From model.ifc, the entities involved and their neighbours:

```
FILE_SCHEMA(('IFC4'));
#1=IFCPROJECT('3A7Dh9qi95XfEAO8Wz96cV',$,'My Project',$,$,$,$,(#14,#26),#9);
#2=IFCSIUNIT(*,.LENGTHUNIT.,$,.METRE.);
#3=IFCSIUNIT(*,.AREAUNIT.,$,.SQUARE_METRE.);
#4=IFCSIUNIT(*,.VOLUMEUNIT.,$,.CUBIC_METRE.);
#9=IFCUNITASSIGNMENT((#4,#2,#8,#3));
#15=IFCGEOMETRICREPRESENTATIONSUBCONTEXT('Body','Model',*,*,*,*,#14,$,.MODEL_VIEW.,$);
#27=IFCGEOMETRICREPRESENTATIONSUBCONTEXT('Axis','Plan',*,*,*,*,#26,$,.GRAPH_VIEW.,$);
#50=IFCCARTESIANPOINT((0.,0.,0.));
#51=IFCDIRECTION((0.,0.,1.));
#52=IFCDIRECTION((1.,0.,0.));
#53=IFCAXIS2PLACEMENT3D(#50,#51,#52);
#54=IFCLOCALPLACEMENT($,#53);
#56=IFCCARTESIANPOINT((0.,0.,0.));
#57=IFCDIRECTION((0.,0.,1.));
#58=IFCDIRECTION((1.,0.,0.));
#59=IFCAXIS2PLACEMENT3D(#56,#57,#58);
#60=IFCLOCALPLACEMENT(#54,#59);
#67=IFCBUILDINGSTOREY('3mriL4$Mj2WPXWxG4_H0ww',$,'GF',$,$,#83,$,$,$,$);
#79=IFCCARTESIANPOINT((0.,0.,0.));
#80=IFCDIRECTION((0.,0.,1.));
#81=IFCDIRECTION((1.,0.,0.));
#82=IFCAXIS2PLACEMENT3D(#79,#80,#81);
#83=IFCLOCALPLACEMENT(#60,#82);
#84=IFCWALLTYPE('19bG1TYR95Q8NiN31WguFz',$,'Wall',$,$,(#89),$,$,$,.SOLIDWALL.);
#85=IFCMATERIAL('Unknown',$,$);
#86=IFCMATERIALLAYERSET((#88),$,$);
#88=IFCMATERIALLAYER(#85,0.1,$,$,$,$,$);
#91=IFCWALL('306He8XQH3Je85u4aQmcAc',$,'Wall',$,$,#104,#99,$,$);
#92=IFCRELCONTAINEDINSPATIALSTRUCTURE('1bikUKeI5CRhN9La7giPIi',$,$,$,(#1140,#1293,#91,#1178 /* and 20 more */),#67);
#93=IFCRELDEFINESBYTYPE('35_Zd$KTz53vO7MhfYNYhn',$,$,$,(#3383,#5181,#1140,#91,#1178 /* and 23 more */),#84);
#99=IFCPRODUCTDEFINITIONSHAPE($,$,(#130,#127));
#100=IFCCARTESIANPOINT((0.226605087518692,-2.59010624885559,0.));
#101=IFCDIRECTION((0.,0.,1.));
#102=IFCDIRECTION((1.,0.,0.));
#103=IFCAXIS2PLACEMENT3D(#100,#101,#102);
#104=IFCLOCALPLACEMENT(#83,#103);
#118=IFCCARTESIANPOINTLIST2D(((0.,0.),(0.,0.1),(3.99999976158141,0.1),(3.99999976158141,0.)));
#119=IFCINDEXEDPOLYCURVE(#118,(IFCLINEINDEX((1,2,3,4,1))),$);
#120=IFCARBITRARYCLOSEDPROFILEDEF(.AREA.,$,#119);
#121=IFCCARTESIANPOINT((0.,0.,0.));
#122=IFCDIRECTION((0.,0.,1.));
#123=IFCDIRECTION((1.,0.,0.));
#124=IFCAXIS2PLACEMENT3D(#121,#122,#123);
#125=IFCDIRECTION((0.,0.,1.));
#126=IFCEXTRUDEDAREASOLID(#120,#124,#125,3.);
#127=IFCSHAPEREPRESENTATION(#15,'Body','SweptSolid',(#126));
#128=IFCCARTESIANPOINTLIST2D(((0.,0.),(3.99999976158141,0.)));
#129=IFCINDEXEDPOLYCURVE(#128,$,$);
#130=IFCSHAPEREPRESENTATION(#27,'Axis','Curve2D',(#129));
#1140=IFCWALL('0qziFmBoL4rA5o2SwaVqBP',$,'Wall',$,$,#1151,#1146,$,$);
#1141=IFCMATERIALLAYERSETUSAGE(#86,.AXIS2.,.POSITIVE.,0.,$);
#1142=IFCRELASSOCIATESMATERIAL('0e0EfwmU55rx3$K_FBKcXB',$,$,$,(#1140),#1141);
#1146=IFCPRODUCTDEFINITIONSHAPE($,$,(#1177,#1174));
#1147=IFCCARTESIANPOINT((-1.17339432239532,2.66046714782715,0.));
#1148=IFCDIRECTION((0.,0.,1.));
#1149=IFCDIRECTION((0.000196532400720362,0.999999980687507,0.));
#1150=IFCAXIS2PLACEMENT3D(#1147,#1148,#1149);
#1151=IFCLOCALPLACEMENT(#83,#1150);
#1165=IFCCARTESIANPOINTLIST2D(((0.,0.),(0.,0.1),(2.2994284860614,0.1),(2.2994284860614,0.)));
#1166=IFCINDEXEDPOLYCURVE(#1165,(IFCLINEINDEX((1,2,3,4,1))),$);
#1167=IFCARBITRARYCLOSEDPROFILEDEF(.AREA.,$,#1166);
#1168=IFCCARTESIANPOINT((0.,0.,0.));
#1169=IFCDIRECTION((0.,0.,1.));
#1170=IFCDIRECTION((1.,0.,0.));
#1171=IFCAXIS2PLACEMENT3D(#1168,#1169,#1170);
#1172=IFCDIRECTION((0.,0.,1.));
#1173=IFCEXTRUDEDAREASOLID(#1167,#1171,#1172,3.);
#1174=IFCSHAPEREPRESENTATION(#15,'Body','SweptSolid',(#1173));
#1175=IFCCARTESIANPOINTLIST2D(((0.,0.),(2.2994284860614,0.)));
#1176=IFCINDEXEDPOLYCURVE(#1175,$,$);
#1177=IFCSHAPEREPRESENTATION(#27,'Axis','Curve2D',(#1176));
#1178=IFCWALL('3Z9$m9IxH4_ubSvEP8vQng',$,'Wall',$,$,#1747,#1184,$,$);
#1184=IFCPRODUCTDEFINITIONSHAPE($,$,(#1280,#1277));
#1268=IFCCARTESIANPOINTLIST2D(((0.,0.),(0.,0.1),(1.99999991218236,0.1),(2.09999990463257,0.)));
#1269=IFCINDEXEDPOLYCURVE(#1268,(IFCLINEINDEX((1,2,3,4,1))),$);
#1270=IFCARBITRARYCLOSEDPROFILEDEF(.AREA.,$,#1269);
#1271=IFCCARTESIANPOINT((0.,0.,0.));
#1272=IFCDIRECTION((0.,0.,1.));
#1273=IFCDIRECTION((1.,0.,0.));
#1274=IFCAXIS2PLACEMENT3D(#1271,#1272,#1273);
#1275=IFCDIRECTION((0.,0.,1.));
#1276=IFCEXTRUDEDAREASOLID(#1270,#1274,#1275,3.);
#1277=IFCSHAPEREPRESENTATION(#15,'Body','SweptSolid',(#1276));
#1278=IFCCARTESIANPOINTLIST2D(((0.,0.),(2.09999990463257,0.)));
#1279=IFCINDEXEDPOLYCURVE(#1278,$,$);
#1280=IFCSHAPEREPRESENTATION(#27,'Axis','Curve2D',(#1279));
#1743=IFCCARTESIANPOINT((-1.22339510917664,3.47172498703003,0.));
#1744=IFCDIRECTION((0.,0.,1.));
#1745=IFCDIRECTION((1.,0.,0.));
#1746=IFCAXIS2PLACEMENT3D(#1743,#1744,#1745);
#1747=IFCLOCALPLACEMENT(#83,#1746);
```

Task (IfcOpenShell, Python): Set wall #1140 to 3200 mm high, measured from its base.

```python
import ifcopenshell
import ifcopenshell.geom
import ifcopenshell.util.representation
import ifcopenshell.util.shape

model = ifcopenshell.open("model.ifc")
settings = ifcopenshell.geom.settings()


def volume(element):
    """Net volume in cubic metres, openings subtracted."""
    shape = ifcopenshell.geom.create_shape(settings, element)
    return ifcopenshell.util.shape.get_volume(shape.geometry)


wall = model.by_guid("0qziFmBoL4rA5o2SwaVqBP")
before = volume(wall)

body = ifcopenshell.util.representation.get_representation(wall, "Model", "Body")
solid = body.Items[0]
old_height = solid.Depth
solid.Depth = 3.2
after = volume(wall)

print(f"height {old_height:g} -> {solid.Depth:g}, volume {before:.3f} -> {after:.3f} m3")

model.write("model_rev.ifc")
```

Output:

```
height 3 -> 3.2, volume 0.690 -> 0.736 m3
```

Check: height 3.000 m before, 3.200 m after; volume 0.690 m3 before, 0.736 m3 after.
